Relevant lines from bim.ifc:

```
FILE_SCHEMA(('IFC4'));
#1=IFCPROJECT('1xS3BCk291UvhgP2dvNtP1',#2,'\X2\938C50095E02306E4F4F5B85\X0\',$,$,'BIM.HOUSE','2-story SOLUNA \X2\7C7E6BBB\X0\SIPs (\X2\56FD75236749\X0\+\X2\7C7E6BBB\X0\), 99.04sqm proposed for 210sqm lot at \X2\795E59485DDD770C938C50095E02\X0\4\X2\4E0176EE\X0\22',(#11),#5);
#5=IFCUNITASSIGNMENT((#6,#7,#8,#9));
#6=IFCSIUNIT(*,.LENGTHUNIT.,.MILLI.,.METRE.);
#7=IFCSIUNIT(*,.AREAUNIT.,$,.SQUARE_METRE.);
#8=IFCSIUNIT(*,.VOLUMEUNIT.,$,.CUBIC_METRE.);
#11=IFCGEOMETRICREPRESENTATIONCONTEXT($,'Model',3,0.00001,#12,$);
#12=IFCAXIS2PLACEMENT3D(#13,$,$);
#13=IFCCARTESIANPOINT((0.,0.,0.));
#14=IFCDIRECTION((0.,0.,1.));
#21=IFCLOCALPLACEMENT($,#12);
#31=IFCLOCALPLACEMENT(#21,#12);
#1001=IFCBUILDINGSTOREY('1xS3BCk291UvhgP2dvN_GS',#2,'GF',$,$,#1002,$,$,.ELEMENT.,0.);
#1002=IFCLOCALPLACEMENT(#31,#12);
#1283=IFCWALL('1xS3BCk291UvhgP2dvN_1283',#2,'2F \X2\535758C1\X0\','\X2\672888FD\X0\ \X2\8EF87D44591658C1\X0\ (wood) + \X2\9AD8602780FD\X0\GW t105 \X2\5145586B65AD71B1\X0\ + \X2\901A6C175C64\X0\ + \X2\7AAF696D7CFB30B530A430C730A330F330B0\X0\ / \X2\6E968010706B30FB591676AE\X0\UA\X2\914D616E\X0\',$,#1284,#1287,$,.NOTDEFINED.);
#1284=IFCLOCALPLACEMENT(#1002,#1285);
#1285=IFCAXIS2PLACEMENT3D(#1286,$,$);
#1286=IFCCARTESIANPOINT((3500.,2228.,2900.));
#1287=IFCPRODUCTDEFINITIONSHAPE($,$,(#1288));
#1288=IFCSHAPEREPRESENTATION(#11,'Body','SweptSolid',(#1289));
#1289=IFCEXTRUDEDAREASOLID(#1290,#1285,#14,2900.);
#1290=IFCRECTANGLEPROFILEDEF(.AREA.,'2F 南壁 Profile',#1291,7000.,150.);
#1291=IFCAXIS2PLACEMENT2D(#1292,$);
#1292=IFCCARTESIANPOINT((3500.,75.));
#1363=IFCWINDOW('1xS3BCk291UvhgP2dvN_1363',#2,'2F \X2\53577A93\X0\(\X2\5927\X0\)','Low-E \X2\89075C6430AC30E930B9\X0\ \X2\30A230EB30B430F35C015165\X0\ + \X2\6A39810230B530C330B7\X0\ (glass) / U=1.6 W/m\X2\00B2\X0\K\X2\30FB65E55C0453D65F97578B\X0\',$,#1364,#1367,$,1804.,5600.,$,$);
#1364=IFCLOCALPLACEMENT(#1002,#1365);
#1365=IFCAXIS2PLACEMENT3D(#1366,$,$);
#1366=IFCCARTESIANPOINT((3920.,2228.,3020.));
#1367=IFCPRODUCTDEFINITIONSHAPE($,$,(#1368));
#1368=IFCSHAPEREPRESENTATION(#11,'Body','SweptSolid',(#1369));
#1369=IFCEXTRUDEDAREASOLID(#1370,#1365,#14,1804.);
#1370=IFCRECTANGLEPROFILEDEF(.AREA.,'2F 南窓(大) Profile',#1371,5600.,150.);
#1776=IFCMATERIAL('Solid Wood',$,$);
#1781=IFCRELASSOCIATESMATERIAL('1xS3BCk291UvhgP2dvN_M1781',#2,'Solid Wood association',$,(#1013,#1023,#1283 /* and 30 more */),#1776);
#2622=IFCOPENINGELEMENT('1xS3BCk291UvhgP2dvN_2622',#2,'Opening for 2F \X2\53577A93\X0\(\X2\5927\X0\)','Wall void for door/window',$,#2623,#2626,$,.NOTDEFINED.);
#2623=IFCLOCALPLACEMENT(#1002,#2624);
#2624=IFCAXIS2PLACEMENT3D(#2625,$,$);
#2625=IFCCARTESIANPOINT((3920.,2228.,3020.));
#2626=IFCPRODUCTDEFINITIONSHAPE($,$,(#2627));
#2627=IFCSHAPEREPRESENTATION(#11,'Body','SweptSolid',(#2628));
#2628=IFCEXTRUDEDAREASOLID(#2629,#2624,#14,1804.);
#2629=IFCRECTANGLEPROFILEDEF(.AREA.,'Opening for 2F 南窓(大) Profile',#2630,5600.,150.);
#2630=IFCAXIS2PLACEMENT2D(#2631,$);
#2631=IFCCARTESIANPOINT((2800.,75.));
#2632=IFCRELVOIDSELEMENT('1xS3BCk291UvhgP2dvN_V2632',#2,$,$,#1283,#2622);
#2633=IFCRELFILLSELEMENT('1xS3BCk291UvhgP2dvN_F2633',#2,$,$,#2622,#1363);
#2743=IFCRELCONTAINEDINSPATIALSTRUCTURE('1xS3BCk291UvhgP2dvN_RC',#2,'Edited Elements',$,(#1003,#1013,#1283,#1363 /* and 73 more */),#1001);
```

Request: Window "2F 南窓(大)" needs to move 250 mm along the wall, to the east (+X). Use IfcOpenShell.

```python
import ifcopenshell
import ifcopenshell.api.geometry
import ifcopenshell.util.placement
import ifcopenshell.util.unit

model = ifcopenshell.open("bim.ifc")
unit_scale = ifcopenshell.util.unit.calculate_unit_scale(model)

window = model.by_guid("1xS3BCk291UvhgP2dvN_1363")
opening = window.FillsVoids[0].RelatingOpeningElement
wall = opening.VoidsElements[0].RelatingBuildingElement

wall_matrix = ifcopenshell.util.placement.get_local_placement(wall.ObjectPlacement)
shift = wall_matrix[:3, 0] * 0.25 / unit_scale
before = ifcopenshell.util.placement.get_local_placement(window.ObjectPlacement)[:3, 3].copy()

# The window is not placed relative to its opening, so move both.
for product in (opening, window):
    matrix = ifcopenshell.util.placement.get_local_placement(product.ObjectPlacement)
    matrix[:3, 3] += shift
    ifcopenshell.api.geometry.edit_object_placement(model, product=product, matrix=matrix, is_si=False)

after = ifcopenshell.util.placement.get_local_placement(window.ObjectPlacement)[:3, 3]
print("window moved by", (after - before).round(3) + 0.0)

model.write("bim_rev.ifc")
```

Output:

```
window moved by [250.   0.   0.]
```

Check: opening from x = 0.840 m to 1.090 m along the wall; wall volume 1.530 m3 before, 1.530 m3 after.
